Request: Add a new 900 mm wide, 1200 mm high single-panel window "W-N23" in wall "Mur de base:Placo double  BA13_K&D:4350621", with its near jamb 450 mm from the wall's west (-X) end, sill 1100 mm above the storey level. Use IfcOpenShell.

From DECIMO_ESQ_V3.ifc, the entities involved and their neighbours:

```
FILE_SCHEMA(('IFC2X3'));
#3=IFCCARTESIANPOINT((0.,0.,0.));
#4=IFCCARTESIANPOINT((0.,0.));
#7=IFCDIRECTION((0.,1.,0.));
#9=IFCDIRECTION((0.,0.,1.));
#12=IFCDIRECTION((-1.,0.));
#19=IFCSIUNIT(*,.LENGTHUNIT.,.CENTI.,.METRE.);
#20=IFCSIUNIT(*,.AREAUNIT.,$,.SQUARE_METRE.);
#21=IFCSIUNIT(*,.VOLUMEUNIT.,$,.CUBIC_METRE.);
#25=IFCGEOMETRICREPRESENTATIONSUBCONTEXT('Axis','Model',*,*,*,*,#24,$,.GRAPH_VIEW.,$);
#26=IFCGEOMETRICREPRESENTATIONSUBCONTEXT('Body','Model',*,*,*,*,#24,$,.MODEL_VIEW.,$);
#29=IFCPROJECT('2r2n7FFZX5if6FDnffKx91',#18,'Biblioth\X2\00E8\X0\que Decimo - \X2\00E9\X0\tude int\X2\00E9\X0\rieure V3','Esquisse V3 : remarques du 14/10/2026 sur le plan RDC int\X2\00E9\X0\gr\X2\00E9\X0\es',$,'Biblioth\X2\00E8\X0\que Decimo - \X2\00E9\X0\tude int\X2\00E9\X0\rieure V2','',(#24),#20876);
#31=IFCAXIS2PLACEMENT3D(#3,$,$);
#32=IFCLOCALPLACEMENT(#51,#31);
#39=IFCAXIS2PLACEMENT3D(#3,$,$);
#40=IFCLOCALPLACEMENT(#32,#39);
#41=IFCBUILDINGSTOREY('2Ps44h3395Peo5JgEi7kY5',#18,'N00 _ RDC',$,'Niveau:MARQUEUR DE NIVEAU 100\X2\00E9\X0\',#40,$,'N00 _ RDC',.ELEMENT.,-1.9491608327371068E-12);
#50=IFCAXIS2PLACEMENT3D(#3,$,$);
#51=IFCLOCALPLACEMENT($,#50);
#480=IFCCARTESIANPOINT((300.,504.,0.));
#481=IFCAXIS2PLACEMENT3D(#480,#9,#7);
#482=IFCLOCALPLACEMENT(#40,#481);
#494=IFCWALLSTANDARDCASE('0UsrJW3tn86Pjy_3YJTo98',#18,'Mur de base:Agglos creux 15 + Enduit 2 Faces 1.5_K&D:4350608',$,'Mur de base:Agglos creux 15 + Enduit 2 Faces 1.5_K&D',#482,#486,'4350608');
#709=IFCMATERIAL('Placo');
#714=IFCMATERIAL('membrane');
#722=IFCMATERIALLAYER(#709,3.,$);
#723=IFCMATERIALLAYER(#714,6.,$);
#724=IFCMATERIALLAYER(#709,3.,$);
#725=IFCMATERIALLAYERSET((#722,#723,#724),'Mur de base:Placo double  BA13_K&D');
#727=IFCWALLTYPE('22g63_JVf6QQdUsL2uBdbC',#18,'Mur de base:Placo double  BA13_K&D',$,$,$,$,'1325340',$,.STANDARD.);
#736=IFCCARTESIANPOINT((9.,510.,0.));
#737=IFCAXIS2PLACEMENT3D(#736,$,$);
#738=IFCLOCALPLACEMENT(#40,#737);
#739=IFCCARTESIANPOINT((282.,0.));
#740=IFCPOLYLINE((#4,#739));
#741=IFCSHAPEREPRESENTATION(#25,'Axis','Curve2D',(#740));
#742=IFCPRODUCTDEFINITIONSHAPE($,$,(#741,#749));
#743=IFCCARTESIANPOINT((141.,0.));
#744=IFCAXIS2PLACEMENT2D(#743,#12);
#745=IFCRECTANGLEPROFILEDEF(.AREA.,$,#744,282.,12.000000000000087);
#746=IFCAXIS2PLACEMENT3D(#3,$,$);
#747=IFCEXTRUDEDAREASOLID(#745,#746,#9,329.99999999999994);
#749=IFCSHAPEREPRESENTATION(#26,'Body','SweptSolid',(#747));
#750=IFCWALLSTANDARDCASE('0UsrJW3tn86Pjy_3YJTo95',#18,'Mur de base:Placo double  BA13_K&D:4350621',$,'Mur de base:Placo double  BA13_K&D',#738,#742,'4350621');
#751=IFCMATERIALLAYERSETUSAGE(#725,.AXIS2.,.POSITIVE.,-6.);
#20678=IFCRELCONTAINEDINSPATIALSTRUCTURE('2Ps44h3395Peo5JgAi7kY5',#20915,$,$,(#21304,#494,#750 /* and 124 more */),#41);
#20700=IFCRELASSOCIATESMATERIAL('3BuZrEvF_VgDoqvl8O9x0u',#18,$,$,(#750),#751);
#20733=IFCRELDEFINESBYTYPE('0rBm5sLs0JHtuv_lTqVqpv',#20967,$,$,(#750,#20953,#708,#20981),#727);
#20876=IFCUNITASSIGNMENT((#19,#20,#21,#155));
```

```python
import numpy as np
import ifcopenshell
import ifcopenshell.api.feature
import ifcopenshell.api.geometry
import ifcopenshell.api.root
import ifcopenshell.api.spatial
import ifcopenshell.api.type
import ifcopenshell.geom
import ifcopenshell.util.element
import ifcopenshell.util.placement
import ifcopenshell.util.representation
import ifcopenshell.util.shape
import ifcopenshell.util.unit

model = ifcopenshell.open("DECIMO_ESQ_V3.ifc")
unit_scale = ifcopenshell.util.unit.calculate_unit_scale(model)
settings = ifcopenshell.geom.settings()


def volume(element):
    """Net volume in cubic metres, openings subtracted."""
    shape = ifcopenshell.geom.create_shape(settings, element)
    return ifcopenshell.util.shape.get_volume(shape.geometry)


wall = model.by_guid("0UsrJW3tn86Pjy_3YJTo95")
storey = ifcopenshell.util.element.get_container(wall, ifc_class="IfcBuildingStorey")
context = ifcopenshell.util.representation.get_context(model, "Model", "Body", "MODEL_VIEW")
before = volume(wall)

width, height, from_end, sill = 0.9, 1.2, 0.45, 1.1  # metres

# The wall runs along its own X axis, and the end named is its -X end.
wall_shape = ifcopenshell.geom.create_shape(settings, wall)
x, y, z = ifcopenshell.util.shape.get_vertices(wall_shape.geometry).T
start = x.min() + from_end
face, thickness = float(y.min()), float(y.max() - y.min())
wall_matrix = ifcopenshell.util.placement.get_local_placement(wall.ObjectPlacement)
level = ifcopenshell.util.placement.get_local_placement(storey.ObjectPlacement)[2, 3]


def in_wall(x, y):
    """Placement at x, y metres in the wall's axes, at sill height."""
    matrix = wall_matrix.copy()
    matrix[:, 3] = wall_matrix @ np.array([x / unit_scale, y / unit_scale, 0.0, 1.0])
    matrix[2, 3] = level + sill / unit_scale
    return matrix


# Opening: a box that overshoots both wall faces by 50 mm.
opening = ifcopenshell.api.root.create_entity(model, ifc_class="IfcOpeningElement")
box = ifcopenshell.api.geometry.add_wall_representation(
    model, context=context, length=width, height=height, thickness=thickness + 0.1
)
ifcopenshell.api.geometry.assign_representation(model, product=opening, representation=box)
ifcopenshell.api.geometry.edit_object_placement(model, product=opening, matrix=in_wall(start, face - 0.05), is_si=False)
ifcopenshell.api.feature.add_feature(model, feature=opening, element=wall)

window = ifcopenshell.api.root.create_entity(model, ifc_class="IfcWindow", name="W-N23")
window.OverallWidth, window.OverallHeight = width / unit_scale, height / unit_scale
body = ifcopenshell.api.geometry.add_window_representation(
    model,
    context=context,
    overall_width=window.OverallWidth,
    overall_height=window.OverallHeight,
    partition_type="SINGLE_PANEL",
)
ifcopenshell.api.geometry.assign_representation(model, product=window, representation=body)
ifcopenshell.api.spatial.assign_container(model, products=[window], relating_structure=storey)
fills = ifcopenshell.api.feature.add_filling(model, opening=opening, element=window)
fills.OwnerHistory = window.OwnerHistory  # required in IFC2X3

# IFC2X3 keeps the operation on the window style.
style = ifcopenshell.api.root.create_entity(model, ifc_class="IfcWindowStyle", name="W-N23")
style.OperationType, style.ConstructionType = "SINGLE_PANEL", "NOTDEFINED"
style.ParameterTakesPrecedence = style.Sizeable = False
ifcopenshell.api.type.assign_type(model, related_objects=[window], relating_type=style)

# Centre the window in the wall's thickness.
ifcopenshell.api.geometry.edit_object_placement(model, product=window, matrix=in_wall(start, face), is_si=False)
window_shape = ifcopenshell.geom.create_shape(settings, window)
depth = ifcopenshell.util.shape.get_vertices(window_shape.geometry)[:, 1]
offset = face + thickness / 2 - (depth.min() + depth.max()) / 2
ifcopenshell.api.geometry.edit_object_placement(model, product=window, matrix=in_wall(start, offset), is_si=False)

after = volume(wall)

print(f"wall volume {before:.3f} -> {after:.3f} m3")

model.write("DECIMO_ESQ_V3_updated.ifc")
```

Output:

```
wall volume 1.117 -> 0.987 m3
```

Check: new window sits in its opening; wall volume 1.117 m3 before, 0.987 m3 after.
